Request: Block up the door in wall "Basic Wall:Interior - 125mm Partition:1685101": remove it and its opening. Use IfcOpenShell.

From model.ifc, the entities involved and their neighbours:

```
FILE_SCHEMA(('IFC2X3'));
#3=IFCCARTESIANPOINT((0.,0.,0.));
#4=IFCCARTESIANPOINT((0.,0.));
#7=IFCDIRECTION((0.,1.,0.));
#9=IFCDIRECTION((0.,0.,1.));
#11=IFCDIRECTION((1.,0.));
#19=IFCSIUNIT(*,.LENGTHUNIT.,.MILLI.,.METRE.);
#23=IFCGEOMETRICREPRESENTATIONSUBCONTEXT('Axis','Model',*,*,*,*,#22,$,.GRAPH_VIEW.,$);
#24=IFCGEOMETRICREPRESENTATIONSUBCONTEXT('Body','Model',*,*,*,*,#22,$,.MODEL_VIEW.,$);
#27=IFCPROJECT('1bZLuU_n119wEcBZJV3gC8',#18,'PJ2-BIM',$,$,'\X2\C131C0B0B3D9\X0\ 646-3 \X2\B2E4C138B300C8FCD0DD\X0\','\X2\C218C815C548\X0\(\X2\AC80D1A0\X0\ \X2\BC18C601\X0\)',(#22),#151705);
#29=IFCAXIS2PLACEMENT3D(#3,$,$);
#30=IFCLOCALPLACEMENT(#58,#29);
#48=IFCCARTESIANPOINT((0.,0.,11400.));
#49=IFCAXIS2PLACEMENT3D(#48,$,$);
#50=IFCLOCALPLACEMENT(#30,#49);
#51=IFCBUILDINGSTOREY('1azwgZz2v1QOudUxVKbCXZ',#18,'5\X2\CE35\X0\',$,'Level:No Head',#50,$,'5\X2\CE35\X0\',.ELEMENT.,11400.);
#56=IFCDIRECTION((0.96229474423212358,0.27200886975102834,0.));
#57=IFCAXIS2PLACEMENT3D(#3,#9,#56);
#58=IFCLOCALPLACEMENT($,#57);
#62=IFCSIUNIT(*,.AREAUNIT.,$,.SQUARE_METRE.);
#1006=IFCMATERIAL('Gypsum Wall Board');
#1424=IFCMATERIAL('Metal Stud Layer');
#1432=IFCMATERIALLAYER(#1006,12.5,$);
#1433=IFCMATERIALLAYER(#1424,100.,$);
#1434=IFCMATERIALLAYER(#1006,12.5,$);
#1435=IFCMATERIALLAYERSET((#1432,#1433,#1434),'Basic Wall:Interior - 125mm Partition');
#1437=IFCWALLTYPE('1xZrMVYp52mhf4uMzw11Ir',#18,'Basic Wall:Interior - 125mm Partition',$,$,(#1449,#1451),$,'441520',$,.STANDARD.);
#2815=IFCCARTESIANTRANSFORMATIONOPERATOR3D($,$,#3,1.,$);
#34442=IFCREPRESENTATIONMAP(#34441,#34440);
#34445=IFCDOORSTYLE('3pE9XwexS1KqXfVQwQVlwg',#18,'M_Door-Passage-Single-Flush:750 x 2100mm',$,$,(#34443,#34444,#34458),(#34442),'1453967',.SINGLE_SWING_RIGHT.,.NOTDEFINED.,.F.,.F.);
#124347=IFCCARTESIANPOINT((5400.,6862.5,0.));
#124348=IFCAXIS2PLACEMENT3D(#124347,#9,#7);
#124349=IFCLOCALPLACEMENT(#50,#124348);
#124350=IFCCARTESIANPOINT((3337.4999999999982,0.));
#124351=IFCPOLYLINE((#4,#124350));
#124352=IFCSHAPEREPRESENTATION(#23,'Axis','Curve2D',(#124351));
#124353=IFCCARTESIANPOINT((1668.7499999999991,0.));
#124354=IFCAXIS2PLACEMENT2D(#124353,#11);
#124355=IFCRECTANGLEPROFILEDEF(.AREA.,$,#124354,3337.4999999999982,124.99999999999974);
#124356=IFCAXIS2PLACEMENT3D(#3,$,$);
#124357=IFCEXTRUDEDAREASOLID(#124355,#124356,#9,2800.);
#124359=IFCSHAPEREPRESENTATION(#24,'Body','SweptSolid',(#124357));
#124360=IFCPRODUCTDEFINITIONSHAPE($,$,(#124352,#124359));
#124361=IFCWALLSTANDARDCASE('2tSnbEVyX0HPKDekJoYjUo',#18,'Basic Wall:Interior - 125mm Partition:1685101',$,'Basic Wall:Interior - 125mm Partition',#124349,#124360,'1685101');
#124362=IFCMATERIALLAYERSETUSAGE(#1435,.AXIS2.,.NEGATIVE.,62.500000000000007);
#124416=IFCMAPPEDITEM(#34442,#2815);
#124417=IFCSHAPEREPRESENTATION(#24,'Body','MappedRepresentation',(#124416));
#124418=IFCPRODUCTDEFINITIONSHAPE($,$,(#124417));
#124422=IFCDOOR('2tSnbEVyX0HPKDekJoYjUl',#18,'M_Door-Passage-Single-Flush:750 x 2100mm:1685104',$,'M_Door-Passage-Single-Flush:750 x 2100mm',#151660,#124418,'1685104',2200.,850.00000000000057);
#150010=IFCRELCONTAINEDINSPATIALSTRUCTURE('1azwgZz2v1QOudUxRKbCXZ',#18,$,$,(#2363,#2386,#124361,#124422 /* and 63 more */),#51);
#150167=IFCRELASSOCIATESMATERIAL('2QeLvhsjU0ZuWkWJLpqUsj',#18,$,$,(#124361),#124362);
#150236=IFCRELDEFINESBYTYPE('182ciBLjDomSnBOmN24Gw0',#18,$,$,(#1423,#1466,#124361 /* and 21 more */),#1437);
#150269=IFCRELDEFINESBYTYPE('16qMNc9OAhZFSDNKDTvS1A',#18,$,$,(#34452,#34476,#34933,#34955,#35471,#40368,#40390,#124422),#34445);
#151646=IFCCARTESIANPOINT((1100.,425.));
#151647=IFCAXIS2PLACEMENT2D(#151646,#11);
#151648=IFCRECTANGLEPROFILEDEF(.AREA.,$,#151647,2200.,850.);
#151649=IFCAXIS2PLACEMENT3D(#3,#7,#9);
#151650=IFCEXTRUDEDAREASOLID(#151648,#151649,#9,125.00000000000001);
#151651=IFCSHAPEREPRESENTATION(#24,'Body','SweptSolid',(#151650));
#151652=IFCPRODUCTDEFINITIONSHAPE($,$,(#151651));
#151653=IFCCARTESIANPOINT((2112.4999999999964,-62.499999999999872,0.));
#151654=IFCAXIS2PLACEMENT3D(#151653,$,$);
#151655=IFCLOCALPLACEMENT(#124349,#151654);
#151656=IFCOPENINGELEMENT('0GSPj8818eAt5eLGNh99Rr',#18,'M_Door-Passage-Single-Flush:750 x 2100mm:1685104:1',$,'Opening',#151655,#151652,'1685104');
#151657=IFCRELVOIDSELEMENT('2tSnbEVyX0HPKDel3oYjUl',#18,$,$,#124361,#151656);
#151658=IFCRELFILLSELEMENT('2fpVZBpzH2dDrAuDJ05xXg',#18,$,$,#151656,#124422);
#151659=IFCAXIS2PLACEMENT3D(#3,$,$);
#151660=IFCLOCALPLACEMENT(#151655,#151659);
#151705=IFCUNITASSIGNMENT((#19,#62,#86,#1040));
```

```python
import ifcopenshell
import ifcopenshell.api.feature
import ifcopenshell.api.root
import ifcopenshell.geom
import ifcopenshell.util.shape

model = ifcopenshell.open("model.ifc")
settings = ifcopenshell.geom.settings()


def volume(element):
    """Net volume in cubic metres, openings subtracted."""
    shape = ifcopenshell.geom.create_shape(settings, element)
    return ifcopenshell.util.shape.get_volume(shape.geometry)


door = model.by_guid("2tSnbEVyX0HPKDekJoYjUl")
opening = door.FillsVoids[0].RelatingOpeningElement
wall = opening.VoidsElements[0].RelatingBuildingElement
before = volume(wall)

ifcopenshell.api.root.remove_product(model, product=door)
ifcopenshell.api.feature.remove_feature(model, feature=opening)

after = volume(wall)

print(f"wall volume {before:.3f} -> {after:.3f} m3")

model.write("model_updated.ifc")
```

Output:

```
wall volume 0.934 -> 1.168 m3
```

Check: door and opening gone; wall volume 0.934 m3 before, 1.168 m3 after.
